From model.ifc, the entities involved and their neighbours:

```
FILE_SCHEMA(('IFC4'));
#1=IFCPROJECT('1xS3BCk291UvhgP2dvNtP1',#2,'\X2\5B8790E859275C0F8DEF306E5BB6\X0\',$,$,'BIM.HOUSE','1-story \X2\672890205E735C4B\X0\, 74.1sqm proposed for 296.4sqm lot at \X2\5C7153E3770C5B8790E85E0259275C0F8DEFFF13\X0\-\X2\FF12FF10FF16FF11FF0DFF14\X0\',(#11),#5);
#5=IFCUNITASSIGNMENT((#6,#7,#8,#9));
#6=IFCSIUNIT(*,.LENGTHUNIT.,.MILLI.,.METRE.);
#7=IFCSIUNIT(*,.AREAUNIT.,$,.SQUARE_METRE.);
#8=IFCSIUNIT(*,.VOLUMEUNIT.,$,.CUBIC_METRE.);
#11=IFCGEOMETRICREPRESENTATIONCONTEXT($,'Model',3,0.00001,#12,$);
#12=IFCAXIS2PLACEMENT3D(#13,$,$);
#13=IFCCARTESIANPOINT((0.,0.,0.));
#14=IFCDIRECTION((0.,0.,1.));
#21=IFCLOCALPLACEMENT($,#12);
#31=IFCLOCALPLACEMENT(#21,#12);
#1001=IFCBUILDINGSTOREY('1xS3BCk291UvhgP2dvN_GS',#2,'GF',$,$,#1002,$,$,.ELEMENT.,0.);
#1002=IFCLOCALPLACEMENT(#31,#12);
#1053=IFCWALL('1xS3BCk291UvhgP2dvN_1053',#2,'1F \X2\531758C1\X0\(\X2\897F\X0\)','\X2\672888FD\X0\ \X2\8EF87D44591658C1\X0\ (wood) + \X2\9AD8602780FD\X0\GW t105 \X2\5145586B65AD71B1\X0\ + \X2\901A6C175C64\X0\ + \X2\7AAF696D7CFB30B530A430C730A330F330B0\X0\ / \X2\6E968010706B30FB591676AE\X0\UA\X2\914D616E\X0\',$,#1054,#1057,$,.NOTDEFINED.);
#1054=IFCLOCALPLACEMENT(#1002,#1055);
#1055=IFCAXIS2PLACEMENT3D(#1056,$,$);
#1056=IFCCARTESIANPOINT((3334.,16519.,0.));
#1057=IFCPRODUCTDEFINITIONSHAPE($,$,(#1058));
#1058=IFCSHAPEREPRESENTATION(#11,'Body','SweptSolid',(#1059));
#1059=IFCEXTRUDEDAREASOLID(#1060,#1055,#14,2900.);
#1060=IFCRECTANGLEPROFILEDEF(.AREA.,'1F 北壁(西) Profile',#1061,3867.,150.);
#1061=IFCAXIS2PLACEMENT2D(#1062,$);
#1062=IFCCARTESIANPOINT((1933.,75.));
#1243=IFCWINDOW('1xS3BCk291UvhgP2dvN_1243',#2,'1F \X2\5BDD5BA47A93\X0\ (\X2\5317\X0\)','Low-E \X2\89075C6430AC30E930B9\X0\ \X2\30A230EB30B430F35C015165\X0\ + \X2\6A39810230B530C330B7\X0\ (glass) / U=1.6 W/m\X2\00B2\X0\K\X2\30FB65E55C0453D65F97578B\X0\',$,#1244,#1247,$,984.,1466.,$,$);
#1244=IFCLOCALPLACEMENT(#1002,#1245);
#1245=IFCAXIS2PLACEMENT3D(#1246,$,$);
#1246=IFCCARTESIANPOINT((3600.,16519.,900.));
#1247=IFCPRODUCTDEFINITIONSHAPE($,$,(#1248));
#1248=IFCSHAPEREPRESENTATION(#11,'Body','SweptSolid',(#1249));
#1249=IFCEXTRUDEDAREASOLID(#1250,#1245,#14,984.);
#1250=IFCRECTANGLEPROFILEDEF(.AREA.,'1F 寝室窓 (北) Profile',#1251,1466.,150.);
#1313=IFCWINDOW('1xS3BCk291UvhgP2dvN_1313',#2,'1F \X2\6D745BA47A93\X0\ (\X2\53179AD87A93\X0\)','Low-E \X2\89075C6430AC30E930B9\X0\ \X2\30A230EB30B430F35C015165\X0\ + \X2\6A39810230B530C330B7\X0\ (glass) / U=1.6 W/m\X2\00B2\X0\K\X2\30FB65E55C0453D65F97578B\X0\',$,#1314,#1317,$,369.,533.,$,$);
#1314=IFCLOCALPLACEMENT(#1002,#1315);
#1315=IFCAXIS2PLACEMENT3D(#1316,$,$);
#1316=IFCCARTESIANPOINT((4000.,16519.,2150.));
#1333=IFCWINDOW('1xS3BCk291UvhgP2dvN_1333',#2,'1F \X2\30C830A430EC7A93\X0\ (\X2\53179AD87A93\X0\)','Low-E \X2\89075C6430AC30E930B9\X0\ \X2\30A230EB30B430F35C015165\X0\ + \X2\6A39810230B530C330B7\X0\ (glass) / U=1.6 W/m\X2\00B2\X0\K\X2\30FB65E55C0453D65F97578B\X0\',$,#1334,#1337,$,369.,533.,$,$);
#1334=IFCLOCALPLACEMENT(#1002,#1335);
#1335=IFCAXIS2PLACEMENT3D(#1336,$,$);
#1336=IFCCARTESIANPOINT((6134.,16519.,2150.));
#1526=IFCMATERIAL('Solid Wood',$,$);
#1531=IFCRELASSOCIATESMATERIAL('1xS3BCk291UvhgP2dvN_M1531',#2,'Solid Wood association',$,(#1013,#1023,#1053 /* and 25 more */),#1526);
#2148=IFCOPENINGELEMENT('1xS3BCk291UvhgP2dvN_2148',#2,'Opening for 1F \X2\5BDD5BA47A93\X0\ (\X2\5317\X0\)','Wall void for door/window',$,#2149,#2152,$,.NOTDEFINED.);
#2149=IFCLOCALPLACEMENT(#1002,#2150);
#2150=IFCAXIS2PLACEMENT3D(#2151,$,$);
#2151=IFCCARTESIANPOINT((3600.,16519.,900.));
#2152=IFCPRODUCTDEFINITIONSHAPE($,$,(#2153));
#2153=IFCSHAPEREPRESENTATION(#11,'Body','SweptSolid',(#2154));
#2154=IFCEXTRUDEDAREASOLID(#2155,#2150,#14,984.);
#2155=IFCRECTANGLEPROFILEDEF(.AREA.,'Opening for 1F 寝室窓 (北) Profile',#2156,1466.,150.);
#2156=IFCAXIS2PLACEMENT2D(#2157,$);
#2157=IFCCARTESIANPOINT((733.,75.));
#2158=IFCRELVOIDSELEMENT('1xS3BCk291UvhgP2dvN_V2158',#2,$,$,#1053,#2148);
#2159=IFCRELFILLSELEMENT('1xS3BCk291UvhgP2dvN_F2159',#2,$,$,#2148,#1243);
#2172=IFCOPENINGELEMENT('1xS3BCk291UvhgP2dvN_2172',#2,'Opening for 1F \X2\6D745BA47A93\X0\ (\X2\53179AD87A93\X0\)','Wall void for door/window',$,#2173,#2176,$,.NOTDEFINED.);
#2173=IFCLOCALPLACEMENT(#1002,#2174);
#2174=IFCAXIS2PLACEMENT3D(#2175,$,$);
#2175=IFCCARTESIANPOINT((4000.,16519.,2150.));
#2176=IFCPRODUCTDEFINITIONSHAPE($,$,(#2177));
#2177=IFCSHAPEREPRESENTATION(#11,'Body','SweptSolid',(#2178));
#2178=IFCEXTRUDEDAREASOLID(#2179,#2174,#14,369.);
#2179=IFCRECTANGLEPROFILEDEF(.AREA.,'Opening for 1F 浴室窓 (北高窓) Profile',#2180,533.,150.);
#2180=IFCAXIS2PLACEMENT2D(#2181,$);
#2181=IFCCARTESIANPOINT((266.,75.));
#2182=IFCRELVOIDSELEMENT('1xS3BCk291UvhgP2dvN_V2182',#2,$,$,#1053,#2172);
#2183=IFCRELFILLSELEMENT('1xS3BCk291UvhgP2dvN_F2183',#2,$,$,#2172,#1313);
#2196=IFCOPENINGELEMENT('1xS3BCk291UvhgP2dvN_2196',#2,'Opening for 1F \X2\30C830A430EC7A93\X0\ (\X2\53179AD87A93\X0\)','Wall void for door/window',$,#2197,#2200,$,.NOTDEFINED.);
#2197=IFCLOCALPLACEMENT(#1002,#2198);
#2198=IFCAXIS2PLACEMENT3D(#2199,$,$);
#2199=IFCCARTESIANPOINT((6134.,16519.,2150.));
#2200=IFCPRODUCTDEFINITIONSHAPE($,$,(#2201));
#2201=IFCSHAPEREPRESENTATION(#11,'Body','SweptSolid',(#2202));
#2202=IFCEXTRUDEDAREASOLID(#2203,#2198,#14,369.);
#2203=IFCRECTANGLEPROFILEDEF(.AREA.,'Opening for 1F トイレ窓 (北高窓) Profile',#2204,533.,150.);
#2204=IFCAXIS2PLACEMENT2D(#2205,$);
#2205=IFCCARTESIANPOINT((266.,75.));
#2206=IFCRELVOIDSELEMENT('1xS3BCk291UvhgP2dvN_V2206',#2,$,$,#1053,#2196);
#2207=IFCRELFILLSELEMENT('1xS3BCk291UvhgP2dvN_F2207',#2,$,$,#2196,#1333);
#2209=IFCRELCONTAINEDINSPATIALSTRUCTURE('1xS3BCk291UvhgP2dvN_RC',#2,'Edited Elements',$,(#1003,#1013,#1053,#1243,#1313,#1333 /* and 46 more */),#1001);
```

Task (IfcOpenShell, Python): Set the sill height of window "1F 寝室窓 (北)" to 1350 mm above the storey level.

```python
import numpy as np
import ifcopenshell
import ifcopenshell.api.geometry
import ifcopenshell.geom
import ifcopenshell.util.element
import ifcopenshell.util.placement
import ifcopenshell.util.shape
import ifcopenshell.util.unit

model = ifcopenshell.open("model.ifc")
unit_scale = ifcopenshell.util.unit.calculate_unit_scale(model)

window = model.by_guid("1xS3BCk291UvhgP2dvN_1243")
opening = window.FillsVoids[0].RelatingOpeningElement
storey = ifcopenshell.util.element.get_container(window, ifc_class="IfcBuildingStorey")
level = ifcopenshell.util.placement.get_local_placement(storey.ObjectPlacement)[2, 3]

# The opening's origin need not be at the sill, so measure its lowest point.
shape = ifcopenshell.geom.create_shape(ifcopenshell.geom.settings(), opening)
bottom = ifcopenshell.util.shape.get_shape_bottom_elevation(shape, shape.geometry) / unit_scale
dz = level + 1.35 / unit_scale - bottom

shift = np.array([0.0, 0.0, dz])
# The window is not placed relative to its opening, so move both.
for product in (opening, window):
    matrix = ifcopenshell.util.placement.get_local_placement(product.ObjectPlacement)
    matrix[:3, 3] += shift
    ifcopenshell.api.geometry.edit_object_placement(model, product=product, matrix=matrix, is_si=False)

print(f"moved by {dz * unit_scale:+.3f} m")

model.write("model_updated.ifc")
```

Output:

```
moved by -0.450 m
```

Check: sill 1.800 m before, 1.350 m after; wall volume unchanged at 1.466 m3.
